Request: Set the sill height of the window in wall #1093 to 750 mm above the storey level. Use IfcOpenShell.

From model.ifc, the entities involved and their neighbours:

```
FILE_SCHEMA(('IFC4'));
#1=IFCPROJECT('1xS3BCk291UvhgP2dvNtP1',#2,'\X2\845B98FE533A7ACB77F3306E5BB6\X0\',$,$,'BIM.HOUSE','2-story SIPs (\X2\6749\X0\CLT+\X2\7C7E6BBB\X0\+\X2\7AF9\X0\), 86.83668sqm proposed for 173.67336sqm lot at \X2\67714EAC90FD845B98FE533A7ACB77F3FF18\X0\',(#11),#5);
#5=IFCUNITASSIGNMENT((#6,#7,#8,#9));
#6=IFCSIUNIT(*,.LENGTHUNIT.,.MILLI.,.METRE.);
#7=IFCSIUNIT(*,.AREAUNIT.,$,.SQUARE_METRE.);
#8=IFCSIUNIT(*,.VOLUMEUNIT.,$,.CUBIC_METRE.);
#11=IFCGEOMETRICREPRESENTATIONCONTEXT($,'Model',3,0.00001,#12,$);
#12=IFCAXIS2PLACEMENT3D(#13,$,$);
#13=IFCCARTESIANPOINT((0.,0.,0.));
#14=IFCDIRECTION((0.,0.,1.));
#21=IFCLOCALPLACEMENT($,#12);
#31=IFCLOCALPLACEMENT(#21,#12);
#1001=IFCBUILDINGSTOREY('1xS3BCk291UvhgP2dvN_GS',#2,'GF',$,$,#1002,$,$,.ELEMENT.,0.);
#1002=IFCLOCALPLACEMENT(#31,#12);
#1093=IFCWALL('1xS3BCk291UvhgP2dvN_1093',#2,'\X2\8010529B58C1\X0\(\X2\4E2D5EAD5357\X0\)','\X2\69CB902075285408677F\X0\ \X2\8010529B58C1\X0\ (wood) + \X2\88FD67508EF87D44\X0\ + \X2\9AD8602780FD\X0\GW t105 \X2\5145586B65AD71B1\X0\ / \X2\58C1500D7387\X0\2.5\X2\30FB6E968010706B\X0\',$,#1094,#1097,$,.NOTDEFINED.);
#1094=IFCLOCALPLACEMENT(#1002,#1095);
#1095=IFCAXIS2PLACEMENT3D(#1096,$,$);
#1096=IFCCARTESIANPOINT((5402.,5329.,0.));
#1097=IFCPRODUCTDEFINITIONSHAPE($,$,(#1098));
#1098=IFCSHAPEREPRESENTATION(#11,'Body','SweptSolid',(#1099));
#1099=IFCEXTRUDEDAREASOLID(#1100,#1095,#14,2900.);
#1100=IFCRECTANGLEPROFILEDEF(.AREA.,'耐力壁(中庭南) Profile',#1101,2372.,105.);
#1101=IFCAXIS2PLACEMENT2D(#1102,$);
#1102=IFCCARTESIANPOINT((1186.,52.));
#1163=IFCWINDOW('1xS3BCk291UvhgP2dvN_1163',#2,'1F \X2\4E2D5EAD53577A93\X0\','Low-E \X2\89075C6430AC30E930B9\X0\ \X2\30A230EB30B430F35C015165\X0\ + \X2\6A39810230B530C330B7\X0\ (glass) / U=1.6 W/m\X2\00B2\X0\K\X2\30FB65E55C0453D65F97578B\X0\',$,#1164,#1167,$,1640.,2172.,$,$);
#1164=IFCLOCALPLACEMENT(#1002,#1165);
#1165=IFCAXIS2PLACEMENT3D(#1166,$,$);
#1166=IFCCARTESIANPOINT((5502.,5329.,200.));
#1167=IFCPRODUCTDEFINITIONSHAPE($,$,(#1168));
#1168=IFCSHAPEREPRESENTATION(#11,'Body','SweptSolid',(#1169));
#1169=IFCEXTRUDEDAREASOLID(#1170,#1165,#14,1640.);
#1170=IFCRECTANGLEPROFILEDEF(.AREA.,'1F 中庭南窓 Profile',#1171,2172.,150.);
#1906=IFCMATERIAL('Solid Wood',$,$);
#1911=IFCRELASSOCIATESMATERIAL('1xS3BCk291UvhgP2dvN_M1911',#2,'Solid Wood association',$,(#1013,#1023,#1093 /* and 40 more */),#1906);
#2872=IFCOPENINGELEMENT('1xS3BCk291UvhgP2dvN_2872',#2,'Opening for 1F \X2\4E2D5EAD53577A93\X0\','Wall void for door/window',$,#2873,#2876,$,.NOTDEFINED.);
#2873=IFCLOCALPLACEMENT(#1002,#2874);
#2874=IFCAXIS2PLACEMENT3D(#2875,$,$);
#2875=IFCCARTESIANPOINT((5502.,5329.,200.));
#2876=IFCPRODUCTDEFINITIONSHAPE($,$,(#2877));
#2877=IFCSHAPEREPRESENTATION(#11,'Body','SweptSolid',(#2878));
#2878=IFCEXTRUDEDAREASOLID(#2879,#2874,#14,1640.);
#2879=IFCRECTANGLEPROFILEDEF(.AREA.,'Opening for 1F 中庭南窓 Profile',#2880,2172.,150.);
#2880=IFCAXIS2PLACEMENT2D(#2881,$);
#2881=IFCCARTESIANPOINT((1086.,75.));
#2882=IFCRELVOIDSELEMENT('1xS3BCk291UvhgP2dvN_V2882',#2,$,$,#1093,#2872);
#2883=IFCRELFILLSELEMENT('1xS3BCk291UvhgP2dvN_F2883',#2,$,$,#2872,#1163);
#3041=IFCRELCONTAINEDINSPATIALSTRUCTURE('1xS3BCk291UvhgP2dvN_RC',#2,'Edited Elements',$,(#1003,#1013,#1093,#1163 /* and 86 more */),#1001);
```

```python
import numpy as np
import ifcopenshell
import ifcopenshell.api.geometry
import ifcopenshell.geom
import ifcopenshell.util.element
import ifcopenshell.util.placement
import ifcopenshell.util.shape
import ifcopenshell.util.unit

model = ifcopenshell.open("model.ifc")
unit_scale = ifcopenshell.util.unit.calculate_unit_scale(model)

window = model.by_guid("1xS3BCk291UvhgP2dvN_1163")
opening = window.FillsVoids[0].RelatingOpeningElement
storey = ifcopenshell.util.element.get_container(window, ifc_class="IfcBuildingStorey")
level = ifcopenshell.util.placement.get_local_placement(storey.ObjectPlacement)[2, 3]

# The opening's origin need not be at the sill, so measure its lowest point.
shape = ifcopenshell.geom.create_shape(ifcopenshell.geom.settings(), opening)
bottom = ifcopenshell.util.shape.get_shape_bottom_elevation(shape, shape.geometry) / unit_scale
dz = level + 0.75 / unit_scale - bottom

shift = np.array([0.0, 0.0, dz])
# The window is not placed relative to its opening, so move both.
for product in (opening, window):
    matrix = ifcopenshell.util.placement.get_local_placement(product.ObjectPlacement)
    matrix[:3, 3] += shift
    ifcopenshell.api.geometry.edit_object_placement(model, product=product, matrix=matrix, is_si=False)

print(f"moved by {dz * unit_scale:+.3f} m")

model.write("model_updated.ifc")
```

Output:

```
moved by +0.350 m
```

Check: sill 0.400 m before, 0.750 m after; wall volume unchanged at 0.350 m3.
